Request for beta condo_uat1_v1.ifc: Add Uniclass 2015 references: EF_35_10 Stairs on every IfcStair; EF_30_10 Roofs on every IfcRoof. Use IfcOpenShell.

First a look at what the model holds.

```python
import ifcopenshell

model = ifcopenshell.open("beta condo_uat1_v1.ifc")
print(model.schema)
print("classifications:", [c.Name for c in model.by_type("IfcClassification")])
for ifc_class in ("IfcDoor", "IfcRoof", "IfcStair", "IfcWall", "IfcWindow"):
    print(ifc_class, len(model.by_type(ifc_class)))
```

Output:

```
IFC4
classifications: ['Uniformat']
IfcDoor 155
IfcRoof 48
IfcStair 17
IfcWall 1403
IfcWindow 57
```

```python
import ifcopenshell
import ifcopenshell.api.classification

model = ifcopenshell.open("beta condo_uat1_v1.ifc")

system = ifcopenshell.api.classification.add_classification(model, classification="Uniclass 2015")

codes = {
    "IfcStair": ("EF_35_10", "Stairs"),
    "IfcRoof": ("EF_30_10", "Roofs"),
}
for ifc_class, (code, name) in codes.items():
    products = model.by_type(ifc_class)
    ifcopenshell.api.classification.add_reference(
        model, products=products, classification=system, identification=code, name=name
    )
    print(code, len(products))

model.write("beta condo_uat1_v1_v2.ifc")
```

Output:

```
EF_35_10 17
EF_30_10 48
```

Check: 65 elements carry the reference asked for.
